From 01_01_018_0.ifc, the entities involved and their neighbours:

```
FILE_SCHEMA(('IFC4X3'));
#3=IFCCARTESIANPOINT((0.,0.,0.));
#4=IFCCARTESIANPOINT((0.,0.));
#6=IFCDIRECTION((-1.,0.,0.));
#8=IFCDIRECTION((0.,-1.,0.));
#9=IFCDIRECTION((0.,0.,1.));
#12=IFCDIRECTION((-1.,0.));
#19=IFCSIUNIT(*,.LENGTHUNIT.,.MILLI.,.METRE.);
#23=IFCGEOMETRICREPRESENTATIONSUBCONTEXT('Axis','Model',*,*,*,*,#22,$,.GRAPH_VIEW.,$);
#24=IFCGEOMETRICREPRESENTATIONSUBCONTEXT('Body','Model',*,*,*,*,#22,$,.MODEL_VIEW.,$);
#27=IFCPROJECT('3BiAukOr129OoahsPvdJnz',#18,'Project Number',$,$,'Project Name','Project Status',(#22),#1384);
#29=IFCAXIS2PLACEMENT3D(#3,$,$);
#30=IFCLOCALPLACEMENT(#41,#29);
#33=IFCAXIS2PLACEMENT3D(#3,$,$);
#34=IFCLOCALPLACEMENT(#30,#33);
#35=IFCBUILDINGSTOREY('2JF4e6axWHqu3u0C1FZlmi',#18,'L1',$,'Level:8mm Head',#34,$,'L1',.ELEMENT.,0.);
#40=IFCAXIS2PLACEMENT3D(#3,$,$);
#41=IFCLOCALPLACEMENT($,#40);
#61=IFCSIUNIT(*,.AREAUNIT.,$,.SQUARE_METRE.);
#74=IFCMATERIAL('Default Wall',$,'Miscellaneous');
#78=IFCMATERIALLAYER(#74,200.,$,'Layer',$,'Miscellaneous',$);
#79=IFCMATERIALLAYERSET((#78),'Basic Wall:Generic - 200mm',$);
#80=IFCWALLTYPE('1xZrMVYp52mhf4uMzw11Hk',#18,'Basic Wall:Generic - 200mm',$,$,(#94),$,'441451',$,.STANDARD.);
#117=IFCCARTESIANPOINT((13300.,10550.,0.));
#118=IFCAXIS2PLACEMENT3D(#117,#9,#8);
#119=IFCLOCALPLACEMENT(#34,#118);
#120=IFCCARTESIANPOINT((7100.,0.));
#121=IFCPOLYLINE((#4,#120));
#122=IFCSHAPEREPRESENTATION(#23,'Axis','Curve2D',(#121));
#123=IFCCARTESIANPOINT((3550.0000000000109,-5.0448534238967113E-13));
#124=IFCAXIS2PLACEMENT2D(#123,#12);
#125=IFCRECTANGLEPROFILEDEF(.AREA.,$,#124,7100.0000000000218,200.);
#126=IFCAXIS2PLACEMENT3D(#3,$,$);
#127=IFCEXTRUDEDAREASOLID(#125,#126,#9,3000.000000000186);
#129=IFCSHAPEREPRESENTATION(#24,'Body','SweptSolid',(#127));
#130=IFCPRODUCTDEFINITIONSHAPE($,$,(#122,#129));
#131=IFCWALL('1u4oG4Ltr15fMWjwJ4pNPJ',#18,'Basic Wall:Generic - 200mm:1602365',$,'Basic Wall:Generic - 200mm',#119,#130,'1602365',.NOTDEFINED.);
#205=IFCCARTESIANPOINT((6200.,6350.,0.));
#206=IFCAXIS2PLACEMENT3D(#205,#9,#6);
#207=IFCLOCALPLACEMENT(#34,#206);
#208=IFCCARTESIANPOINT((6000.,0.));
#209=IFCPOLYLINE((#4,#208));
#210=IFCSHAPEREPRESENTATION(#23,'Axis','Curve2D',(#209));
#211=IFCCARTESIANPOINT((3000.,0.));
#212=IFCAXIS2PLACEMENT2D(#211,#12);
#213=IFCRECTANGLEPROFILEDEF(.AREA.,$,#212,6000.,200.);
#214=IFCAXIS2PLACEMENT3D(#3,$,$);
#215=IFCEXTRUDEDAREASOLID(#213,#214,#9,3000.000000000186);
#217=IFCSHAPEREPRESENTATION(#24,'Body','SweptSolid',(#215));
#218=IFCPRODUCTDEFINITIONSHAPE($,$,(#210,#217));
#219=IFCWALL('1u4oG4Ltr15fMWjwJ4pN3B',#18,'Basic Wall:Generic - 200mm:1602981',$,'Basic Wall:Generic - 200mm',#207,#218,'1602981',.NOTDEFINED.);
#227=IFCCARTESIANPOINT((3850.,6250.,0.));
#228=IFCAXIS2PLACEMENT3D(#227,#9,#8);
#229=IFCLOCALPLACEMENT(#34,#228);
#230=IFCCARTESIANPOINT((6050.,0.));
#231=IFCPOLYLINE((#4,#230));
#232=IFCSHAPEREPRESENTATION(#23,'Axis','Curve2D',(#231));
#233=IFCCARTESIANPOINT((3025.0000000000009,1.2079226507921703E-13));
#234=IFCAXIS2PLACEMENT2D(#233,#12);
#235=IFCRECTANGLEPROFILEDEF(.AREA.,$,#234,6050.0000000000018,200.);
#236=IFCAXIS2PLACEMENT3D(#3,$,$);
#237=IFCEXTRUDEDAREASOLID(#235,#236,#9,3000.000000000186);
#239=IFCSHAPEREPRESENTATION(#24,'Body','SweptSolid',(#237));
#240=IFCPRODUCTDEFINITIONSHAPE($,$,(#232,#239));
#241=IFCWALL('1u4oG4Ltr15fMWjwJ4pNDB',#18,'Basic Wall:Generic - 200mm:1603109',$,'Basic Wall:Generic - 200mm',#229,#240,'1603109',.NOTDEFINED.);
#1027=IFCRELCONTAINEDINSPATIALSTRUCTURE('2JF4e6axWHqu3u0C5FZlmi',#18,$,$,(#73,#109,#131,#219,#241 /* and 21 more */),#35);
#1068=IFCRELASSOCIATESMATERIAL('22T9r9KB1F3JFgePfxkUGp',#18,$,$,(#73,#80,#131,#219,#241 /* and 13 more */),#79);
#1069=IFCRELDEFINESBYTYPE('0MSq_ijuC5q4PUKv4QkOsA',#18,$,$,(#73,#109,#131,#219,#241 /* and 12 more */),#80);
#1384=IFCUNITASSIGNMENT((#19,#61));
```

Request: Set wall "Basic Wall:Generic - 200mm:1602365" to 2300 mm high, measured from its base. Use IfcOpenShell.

```python
import ifcopenshell
import ifcopenshell.geom
import ifcopenshell.util.representation
import ifcopenshell.util.shape
import ifcopenshell.util.unit

model = ifcopenshell.open("01_01_018_0.ifc")
unit_scale = ifcopenshell.util.unit.calculate_unit_scale(model)
settings = ifcopenshell.geom.settings()


def volume(element):
    """Net volume in cubic metres, openings subtracted."""
    shape = ifcopenshell.geom.create_shape(settings, element)
    return ifcopenshell.util.shape.get_volume(shape.geometry)


wall = model.by_guid("1u4oG4Ltr15fMWjwJ4pNPJ")
before = volume(wall)

body = ifcopenshell.util.representation.get_representation(wall, "Model", "Body")
solid = body.Items[0]
old_height = solid.Depth
solid.Depth = 2.3 / unit_scale
after = volume(wall)

print(f"height {old_height:g} -> {solid.Depth:g}, volume {before:.3f} -> {after:.3f} m3")

model.write("01_01_018_0_v2.ifc")
```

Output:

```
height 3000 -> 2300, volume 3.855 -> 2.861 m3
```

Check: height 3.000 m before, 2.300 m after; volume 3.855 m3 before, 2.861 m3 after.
